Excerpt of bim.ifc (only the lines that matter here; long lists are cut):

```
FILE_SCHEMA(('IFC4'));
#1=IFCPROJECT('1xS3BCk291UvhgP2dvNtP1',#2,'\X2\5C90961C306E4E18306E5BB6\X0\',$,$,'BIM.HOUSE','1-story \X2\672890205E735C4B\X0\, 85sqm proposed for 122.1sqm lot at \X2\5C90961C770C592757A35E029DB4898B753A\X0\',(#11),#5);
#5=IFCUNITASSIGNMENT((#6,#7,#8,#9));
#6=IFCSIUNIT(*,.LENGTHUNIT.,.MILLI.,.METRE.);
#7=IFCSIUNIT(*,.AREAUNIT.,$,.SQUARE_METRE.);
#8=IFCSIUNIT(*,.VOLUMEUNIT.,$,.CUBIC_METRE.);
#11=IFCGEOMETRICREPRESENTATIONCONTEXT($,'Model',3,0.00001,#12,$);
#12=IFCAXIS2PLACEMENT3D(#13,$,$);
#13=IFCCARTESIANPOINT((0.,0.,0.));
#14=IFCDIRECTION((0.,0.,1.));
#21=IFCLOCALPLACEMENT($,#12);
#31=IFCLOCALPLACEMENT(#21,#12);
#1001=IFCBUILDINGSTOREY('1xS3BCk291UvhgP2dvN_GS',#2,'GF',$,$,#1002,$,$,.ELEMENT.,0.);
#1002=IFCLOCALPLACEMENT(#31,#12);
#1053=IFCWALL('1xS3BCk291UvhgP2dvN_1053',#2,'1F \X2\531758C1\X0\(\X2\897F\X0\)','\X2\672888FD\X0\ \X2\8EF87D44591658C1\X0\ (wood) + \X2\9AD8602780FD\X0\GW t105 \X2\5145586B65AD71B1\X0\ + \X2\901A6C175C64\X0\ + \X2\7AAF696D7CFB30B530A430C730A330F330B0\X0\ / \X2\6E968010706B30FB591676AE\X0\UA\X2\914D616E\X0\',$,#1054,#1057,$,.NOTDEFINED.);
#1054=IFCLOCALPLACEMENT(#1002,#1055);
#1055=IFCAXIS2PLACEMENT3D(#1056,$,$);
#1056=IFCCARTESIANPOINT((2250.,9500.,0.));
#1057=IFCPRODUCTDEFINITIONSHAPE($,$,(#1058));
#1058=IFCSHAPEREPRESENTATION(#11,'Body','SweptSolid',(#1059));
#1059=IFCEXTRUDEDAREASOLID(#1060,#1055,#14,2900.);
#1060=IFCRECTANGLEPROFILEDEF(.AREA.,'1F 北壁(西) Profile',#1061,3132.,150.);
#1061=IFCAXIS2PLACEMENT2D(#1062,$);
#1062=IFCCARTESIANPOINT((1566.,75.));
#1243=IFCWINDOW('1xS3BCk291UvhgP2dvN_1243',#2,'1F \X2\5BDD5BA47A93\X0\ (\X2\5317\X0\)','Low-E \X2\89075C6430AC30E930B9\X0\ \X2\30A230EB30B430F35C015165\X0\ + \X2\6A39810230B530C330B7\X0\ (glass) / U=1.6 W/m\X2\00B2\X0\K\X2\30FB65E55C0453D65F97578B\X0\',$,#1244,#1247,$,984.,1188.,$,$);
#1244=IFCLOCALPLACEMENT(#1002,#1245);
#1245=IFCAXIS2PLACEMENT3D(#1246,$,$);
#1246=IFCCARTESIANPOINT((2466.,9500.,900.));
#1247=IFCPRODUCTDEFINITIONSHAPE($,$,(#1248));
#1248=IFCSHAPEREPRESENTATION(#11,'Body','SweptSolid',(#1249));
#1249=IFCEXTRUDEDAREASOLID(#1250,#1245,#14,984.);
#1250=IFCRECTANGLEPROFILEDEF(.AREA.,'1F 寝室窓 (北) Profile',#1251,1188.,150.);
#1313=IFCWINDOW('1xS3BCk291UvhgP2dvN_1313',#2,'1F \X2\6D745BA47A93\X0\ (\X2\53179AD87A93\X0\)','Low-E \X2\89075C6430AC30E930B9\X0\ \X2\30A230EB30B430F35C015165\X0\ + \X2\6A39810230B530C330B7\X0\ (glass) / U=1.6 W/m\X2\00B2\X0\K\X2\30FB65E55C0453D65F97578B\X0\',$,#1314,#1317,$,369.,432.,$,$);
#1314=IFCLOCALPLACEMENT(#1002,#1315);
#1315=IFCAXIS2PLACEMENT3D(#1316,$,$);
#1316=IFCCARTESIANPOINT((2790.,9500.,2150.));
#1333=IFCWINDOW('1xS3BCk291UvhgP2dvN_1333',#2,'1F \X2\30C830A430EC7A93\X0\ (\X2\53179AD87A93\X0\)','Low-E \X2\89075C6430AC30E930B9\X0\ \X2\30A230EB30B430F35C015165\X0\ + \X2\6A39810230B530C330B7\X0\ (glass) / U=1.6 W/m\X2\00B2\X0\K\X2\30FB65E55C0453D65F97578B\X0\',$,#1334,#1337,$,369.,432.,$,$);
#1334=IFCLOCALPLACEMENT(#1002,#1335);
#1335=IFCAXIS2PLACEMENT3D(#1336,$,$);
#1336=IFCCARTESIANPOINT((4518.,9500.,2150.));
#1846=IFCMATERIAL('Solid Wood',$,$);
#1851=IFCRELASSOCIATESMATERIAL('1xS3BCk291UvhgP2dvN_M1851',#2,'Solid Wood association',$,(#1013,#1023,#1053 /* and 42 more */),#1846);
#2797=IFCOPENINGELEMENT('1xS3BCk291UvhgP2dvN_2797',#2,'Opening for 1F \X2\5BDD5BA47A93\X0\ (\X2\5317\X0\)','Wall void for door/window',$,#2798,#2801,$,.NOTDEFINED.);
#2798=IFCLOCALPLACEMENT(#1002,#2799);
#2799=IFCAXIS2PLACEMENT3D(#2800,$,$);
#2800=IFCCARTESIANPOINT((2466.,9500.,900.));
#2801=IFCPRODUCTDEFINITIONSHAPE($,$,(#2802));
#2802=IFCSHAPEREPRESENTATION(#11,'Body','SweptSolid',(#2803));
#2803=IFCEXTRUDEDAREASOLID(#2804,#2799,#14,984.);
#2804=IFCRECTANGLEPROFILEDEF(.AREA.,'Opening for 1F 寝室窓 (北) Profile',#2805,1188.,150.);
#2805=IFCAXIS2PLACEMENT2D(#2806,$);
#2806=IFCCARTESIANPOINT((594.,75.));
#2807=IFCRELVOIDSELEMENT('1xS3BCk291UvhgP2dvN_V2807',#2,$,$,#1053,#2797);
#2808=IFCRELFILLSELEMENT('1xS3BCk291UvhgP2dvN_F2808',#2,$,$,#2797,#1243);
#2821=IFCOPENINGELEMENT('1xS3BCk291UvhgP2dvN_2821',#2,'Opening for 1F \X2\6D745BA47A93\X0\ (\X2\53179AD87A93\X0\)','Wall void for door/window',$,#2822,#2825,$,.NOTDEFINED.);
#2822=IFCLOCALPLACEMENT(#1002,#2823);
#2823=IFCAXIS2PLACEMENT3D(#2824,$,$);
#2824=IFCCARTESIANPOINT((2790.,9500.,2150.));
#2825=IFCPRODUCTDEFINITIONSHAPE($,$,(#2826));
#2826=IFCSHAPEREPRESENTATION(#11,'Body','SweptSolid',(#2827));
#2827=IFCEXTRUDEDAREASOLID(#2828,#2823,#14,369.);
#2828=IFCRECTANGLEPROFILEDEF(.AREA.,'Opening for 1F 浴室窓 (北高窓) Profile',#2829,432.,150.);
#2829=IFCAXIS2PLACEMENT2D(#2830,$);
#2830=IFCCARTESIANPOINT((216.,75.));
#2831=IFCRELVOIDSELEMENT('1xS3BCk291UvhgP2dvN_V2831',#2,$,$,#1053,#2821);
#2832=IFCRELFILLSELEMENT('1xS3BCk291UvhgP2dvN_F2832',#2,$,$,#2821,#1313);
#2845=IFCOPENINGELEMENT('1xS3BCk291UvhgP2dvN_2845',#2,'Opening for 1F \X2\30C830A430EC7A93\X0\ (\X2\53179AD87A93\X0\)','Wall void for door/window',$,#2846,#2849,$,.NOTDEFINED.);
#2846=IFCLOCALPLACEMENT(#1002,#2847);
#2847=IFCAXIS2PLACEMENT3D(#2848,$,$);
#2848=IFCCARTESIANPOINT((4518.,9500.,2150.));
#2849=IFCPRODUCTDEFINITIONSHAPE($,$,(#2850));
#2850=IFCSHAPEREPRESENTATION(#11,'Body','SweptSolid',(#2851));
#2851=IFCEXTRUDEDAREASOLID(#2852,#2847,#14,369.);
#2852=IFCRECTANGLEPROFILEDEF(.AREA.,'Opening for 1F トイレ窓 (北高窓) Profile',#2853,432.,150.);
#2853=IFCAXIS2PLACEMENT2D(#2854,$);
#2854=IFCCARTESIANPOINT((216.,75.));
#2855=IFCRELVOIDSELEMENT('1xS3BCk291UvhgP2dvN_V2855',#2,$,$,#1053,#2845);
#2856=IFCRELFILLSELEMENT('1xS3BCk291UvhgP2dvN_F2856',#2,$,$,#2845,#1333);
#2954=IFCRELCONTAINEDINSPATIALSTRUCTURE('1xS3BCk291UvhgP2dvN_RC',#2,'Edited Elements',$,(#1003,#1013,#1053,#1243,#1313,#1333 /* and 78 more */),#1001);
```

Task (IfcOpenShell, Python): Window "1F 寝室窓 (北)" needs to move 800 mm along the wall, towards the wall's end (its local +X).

```python
import ifcopenshell
import ifcopenshell.api.geometry
import ifcopenshell.util.placement

model = ifcopenshell.open("bim.ifc")

window = model.by_guid("1xS3BCk291UvhgP2dvN_1243")
opening = window.FillsVoids[0].RelatingOpeningElement
wall = opening.VoidsElements[0].RelatingBuildingElement

wall_matrix = ifcopenshell.util.placement.get_local_placement(wall.ObjectPlacement)
shift = wall_matrix[:3, 0] * 800.0
before = ifcopenshell.util.placement.get_local_placement(window.ObjectPlacement)[:3, 3].copy()

# The window is not placed relative to its opening, so move both.
for product in (opening, window):
    matrix = ifcopenshell.util.placement.get_local_placement(product.ObjectPlacement)
    matrix[:3, 3] += shift
    ifcopenshell.api.geometry.edit_object_placement(model, product=product, matrix=matrix, is_si=False)

after = ifcopenshell.util.placement.get_local_placement(window.ObjectPlacement)[:3, 3]
print("window moved by", (after - before).round(3) + 0.0)

model.write("bim_rev.ifc")
```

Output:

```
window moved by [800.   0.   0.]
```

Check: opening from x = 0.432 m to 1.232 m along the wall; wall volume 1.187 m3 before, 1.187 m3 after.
